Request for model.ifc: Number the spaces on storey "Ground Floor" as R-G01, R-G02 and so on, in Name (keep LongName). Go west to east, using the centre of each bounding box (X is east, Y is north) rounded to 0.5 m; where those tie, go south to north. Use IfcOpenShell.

First a look at what the model holds.

```python
import ifcopenshell
import ifcopenshell.util.element
import ifcopenshell.util.placement

model = ifcopenshell.open("model.ifc")
print(model.schema)
storey = next(s for s in model.by_type("IfcBuildingStorey") if s.Name == "Ground Floor")
spaces = [e for e in ifcopenshell.util.element.get_decomposition(storey) if e.is_a("IfcSpace")]
for e in sorted(spaces, key=lambda e: e.id()):
    origin = ifcopenshell.util.placement.get_local_placement(e.ObjectPlacement)[:3, 3]
    print(e.id(), e.Name, e.LongName, origin.round(2) + 0.0, sep=" | ")
```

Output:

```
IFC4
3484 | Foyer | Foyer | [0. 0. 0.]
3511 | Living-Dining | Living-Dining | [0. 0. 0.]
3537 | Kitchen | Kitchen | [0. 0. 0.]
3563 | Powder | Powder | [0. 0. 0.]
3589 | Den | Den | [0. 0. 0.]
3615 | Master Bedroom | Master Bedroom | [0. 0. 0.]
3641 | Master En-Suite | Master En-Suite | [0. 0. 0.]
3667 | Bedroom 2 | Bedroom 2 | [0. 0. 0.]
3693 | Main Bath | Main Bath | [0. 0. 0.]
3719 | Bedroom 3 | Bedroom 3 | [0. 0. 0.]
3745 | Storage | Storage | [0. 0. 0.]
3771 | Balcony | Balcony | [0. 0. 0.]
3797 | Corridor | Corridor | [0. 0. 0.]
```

```python
import ifcopenshell
import ifcopenshell.geom
import ifcopenshell.util.element
import ifcopenshell.util.shape

model = ifcopenshell.open("model.ifc")
settings = ifcopenshell.geom.settings()
settings.set("use-world-coords", True)


def centre(element):
    shape = ifcopenshell.geom.create_shape(settings, element)
    return ifcopenshell.util.shape.get_bbox_centroid(shape.geometry)


storey = next(s for s in model.by_type("IfcBuildingStorey") if s.Name == "Ground Floor")
spaces = [e for e in ifcopenshell.util.element.get_decomposition(storey) if e.is_a("IfcSpace")]

# Insertion points can sit at a corner or the storey origin, so sort by the geometry (in metres).
centres = {e: centre(e) for e in spaces}
spaces.sort(key=lambda e: (round(centres[e][0] / 0.5), centres[e][1]))

for i, e in enumerate(spaces, start=1):
    number = f"R-G{i:02d}"
    e.Name = number
    print(e.id(), number)

model.write("model_edited.ifc")
```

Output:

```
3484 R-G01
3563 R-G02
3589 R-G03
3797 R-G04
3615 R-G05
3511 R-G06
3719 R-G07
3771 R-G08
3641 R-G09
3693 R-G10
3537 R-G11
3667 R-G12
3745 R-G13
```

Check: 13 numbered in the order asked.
